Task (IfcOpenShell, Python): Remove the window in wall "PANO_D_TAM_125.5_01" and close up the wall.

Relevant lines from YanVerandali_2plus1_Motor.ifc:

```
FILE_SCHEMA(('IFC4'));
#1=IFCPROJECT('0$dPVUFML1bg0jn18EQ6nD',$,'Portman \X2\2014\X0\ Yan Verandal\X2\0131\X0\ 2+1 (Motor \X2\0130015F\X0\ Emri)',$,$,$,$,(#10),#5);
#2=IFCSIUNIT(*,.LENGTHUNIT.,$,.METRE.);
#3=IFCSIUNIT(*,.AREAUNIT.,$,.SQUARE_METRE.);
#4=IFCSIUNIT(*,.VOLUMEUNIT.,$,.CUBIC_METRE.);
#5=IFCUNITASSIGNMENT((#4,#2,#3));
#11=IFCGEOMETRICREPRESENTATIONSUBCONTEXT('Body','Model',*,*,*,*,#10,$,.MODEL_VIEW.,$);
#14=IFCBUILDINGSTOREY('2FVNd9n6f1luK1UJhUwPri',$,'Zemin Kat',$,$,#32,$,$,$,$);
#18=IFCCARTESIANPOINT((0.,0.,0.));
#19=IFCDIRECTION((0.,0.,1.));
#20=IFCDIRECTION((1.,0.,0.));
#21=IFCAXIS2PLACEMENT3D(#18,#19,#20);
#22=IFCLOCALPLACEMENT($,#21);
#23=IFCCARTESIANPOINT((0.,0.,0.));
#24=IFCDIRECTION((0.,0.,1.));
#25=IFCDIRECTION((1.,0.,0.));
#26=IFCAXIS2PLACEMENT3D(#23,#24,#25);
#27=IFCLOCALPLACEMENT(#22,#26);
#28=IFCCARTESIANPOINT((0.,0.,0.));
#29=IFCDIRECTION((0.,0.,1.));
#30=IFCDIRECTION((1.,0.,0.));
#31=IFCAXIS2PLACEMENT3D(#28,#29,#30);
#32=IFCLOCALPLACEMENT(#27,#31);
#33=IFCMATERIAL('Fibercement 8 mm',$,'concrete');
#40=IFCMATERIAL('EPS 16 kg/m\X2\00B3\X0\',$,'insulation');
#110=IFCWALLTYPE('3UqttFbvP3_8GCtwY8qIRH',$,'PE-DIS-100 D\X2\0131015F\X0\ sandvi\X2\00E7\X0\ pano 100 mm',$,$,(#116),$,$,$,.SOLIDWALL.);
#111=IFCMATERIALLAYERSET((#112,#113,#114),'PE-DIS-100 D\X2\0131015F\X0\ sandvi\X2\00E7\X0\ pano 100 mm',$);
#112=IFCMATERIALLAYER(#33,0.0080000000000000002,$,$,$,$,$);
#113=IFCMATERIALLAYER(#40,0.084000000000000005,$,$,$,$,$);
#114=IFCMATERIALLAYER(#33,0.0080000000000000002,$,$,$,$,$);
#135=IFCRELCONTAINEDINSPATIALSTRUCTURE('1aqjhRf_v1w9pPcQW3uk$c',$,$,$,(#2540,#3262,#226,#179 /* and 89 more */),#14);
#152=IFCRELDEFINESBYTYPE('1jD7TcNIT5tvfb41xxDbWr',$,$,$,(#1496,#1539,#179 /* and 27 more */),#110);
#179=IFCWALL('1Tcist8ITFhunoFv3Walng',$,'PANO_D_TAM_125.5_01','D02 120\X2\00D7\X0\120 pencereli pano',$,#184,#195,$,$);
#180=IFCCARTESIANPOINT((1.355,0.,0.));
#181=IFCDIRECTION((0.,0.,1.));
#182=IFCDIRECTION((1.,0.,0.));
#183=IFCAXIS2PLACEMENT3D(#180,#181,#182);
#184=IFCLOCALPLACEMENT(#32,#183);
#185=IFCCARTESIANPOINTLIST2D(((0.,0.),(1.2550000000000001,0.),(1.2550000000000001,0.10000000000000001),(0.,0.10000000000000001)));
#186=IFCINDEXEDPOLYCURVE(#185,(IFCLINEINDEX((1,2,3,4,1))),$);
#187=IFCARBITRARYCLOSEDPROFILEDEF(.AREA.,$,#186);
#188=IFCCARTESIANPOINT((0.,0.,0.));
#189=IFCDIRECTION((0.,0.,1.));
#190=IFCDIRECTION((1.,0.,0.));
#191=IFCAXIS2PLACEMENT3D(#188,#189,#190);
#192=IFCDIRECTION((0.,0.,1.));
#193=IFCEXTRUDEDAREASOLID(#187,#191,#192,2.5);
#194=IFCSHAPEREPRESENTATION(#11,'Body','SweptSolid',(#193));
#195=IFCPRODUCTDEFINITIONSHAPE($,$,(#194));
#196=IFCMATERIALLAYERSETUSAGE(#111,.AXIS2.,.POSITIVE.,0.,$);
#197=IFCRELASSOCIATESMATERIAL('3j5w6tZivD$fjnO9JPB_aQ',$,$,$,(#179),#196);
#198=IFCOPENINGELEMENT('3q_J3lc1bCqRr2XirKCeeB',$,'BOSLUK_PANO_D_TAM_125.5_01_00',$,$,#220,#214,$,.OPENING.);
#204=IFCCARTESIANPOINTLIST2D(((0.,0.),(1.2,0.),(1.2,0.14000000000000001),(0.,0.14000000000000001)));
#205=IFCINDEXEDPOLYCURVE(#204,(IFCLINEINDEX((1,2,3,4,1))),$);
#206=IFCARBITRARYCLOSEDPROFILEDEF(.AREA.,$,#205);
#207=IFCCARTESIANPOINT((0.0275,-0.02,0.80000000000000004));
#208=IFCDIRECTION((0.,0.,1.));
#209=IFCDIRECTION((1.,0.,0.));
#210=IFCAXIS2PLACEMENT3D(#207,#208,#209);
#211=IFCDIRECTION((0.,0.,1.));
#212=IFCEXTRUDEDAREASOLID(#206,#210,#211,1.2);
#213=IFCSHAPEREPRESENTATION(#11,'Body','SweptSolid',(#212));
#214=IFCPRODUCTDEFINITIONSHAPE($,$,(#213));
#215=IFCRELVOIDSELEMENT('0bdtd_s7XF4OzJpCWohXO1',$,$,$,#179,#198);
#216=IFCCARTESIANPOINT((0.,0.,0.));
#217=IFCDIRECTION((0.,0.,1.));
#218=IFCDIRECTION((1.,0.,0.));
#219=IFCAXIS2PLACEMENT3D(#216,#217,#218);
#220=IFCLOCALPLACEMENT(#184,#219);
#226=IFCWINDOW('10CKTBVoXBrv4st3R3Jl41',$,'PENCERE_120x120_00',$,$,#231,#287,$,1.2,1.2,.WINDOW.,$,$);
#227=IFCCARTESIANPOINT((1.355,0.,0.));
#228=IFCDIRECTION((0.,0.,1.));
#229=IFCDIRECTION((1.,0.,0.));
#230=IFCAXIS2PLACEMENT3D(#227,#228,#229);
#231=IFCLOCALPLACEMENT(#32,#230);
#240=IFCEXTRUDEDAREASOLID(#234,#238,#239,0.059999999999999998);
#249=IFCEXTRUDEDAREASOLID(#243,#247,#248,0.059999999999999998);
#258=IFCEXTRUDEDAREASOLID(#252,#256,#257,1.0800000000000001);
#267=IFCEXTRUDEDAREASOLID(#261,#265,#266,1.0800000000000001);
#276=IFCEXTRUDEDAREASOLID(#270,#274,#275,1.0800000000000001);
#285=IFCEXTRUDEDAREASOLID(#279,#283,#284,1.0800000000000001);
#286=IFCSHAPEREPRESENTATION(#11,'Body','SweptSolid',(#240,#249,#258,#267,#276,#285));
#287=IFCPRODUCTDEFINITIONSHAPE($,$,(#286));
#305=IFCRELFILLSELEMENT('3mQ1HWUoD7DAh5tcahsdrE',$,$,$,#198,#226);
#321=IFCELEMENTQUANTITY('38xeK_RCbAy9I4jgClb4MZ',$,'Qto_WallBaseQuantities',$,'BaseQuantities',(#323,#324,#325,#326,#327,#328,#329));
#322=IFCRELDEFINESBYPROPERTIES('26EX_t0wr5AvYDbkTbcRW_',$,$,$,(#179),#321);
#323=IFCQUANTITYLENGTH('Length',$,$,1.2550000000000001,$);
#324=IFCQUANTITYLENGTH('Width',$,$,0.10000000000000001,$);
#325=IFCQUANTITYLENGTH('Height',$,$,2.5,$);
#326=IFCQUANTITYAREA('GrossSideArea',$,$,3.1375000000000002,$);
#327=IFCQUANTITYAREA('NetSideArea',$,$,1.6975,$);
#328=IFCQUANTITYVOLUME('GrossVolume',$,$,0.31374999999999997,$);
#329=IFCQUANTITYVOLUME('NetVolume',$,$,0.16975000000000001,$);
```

```python
import ifcopenshell
import ifcopenshell.api.feature
import ifcopenshell.api.pset
import ifcopenshell.api.root
import ifcopenshell.geom
import ifcopenshell.util.element
import ifcopenshell.util.shape
import ifcopenshell.util.unit

model = ifcopenshell.open("YanVerandali_2plus1_Motor.ifc")
area_scale = ifcopenshell.util.unit.calculate_unit_scale(model, "AREAUNIT")
volume_scale = ifcopenshell.util.unit.calculate_unit_scale(model, "VOLUMEUNIT")
settings = ifcopenshell.geom.settings()


def volume(element):
    """Net volume in cubic metres, openings subtracted."""
    shape = ifcopenshell.geom.create_shape(settings, element)
    return ifcopenshell.util.shape.get_volume(shape.geometry)


window = model.by_id(226)
opening = window.FillsVoids[0].RelatingOpeningElement
wall = opening.VoidsElements[0].RelatingBuildingElement
before = volume(wall)

ifcopenshell.api.root.remove_product(model, product=window)
ifcopenshell.api.feature.remove_feature(model, feature=opening)

after = volume(wall)
thickness = 0.1  # wall thickness in metres

# Update the wall's stored quantities.
qto = model.by_id(ifcopenshell.util.element.get_pset(wall, "Qto_WallBaseQuantities", should_inherit=False)["id"])
ifcopenshell.api.pset.edit_qto(model, qto=qto, properties={
    "NetSideArea": after / thickness / area_scale,
    "NetVolume": after / volume_scale,
})

print(f"wall volume {before:.3f} -> {after:.3f} m3")

model.write("YanVerandali_2plus1_Motor_edited.ifc")
```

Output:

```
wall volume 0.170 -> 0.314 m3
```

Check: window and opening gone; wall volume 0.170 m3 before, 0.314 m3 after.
